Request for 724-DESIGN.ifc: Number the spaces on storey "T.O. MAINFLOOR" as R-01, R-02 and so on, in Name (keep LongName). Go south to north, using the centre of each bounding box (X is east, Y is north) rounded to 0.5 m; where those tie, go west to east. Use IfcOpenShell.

First a look at what the model holds.

```python
import ifcopenshell
import ifcopenshell.util.element
import ifcopenshell.util.placement

model = ifcopenshell.open("724-DESIGN.ifc")
print(model.schema)
storey = next(s for s in model.by_type("IfcBuildingStorey") if s.Name == "T.O. MAINFLOOR")
spaces = [e for e in ifcopenshell.util.element.get_decomposition(storey) if e.is_a("IfcSpace")]
for e in sorted(spaces, key=lambda e: e.id()):
    origin = ifcopenshell.util.placement.get_local_placement(e.ObjectPlacement)[:3, 3]
    print(e.id(), e.Name, e.LongName, origin.round(2) + 0.0, sep=" | ")
```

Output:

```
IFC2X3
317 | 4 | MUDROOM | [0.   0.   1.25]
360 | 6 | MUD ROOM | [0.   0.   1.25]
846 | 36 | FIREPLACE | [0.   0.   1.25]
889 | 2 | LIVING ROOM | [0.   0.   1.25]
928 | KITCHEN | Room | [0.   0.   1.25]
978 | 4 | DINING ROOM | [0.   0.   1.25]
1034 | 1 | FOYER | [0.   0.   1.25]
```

```python
import ifcopenshell
import ifcopenshell.geom
import ifcopenshell.util.element
import ifcopenshell.util.shape

model = ifcopenshell.open("724-DESIGN.ifc")
settings = ifcopenshell.geom.settings()
settings.set("use-world-coords", True)


def centre(element):
    shape = ifcopenshell.geom.create_shape(settings, element)
    return ifcopenshell.util.shape.get_bbox_centroid(shape.geometry)


storey = next(s for s in model.by_type("IfcBuildingStorey") if s.Name == "T.O. MAINFLOOR")
spaces = [e for e in ifcopenshell.util.element.get_decomposition(storey) if e.is_a("IfcSpace")]

# Insertion points can sit at a corner or the storey origin, so sort by the geometry (in metres).
centres = {e: centre(e) for e in spaces}
spaces.sort(key=lambda e: (round(centres[e][1] / 0.5), centres[e][0]))

for i, e in enumerate(spaces, start=1):
    number = f"R-{i:02d}"
    e.Name = number
    print(e.id(), number)

model.write("724-DESIGN_v2.ifc")
```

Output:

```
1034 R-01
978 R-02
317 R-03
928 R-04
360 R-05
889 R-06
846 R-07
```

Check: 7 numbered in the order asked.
